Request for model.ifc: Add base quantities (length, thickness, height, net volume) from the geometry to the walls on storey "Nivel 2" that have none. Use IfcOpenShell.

First a look at what the model holds.

```python
import ifcopenshell
import ifcopenshell.util.element
import ifcopenshell.util.unit

model = ifcopenshell.open("model.ifc")
print(model.schema)
for unit_type in ("LENGTHUNIT", "AREAUNIT", "VOLUMEUNIT"):
    print(unit_type, ifcopenshell.util.unit.calculate_unit_scale(model, unit_type))
storey = next(s for s in model.by_type("IfcBuildingStorey") if s.Name == "Nivel 2")
walls = [e for e in ifcopenshell.util.element.get_decomposition(storey) if e.is_a("IfcWall")]
for e in sorted(walls, key=lambda e: e.id()):
    print(e.id(), e.is_a(), e.Name, list(ifcopenshell.util.element.get_psets(e, qtos_only=True)), sep=" | ")
```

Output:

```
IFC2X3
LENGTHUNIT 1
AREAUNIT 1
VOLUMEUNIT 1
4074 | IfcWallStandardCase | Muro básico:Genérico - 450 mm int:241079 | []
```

```python
import ifcopenshell
import ifcopenshell.api.pset
import ifcopenshell.geom
import ifcopenshell.util.element
import ifcopenshell.util.shape
import ifcopenshell.util.unit

model = ifcopenshell.open("model.ifc")
unit_scale = ifcopenshell.util.unit.calculate_unit_scale(model)
volume_scale = ifcopenshell.util.unit.calculate_unit_scale(model, "VOLUMEUNIT")
settings = ifcopenshell.geom.settings()

storey = next(s for s in model.by_type("IfcBuildingStorey") if s.Name == "Nivel 2")
walls = [e for e in ifcopenshell.util.element.get_decomposition(storey) if e.is_a("IfcWall")]

for e in sorted(walls, key=lambda e: e.id()):
    if ifcopenshell.util.element.get_psets(e, qtos_only=True, should_inherit=False):
        continue
    # Geometry comes back in metres, in the element's own axes.
    shape = ifcopenshell.geom.create_shape(settings, e)
    values = {
        "Length": ifcopenshell.util.shape.get_x(shape.geometry) / unit_scale,
        "Width": ifcopenshell.util.shape.get_y(shape.geometry) / unit_scale,
        "Height": ifcopenshell.util.shape.get_z(shape.geometry) / unit_scale,
        "NetVolume": ifcopenshell.util.shape.get_volume(shape.geometry) / volume_scale,
    }
    qto = ifcopenshell.api.pset.add_qto(model, product=e, name="BaseQuantities")
    ifcopenshell.api.pset.edit_qto(model, qto=qto, properties=values)
    print(e.id(), {k: round(v, 3) for k, v in values.items()})

model.write("model_v2.ifc")
```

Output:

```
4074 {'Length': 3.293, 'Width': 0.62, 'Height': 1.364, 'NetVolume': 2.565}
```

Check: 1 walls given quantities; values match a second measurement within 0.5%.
